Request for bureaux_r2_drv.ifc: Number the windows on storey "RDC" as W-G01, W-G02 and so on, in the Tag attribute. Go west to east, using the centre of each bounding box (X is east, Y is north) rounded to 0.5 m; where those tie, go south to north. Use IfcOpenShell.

First a look at what the model holds.

```python
import ifcopenshell
import ifcopenshell.util.element
import ifcopenshell.util.placement

model = ifcopenshell.open("bureaux_r2_drv.ifc")
print(model.schema)
storey = next(s for s in model.by_type("IfcBuildingStorey") if s.Name == "RDC")
windows = [e for e in ifcopenshell.util.element.get_decomposition(storey) if e.is_a("IfcWindow")]
for e in sorted(windows, key=lambda e: e.id()):
    origin = ifcopenshell.util.placement.get_local_placement(e.ObjectPlacement)[:3, 3]
    print(e.id(), e.Tag, e.Name, origin.round(2) + 0.0, sep=" | ")
```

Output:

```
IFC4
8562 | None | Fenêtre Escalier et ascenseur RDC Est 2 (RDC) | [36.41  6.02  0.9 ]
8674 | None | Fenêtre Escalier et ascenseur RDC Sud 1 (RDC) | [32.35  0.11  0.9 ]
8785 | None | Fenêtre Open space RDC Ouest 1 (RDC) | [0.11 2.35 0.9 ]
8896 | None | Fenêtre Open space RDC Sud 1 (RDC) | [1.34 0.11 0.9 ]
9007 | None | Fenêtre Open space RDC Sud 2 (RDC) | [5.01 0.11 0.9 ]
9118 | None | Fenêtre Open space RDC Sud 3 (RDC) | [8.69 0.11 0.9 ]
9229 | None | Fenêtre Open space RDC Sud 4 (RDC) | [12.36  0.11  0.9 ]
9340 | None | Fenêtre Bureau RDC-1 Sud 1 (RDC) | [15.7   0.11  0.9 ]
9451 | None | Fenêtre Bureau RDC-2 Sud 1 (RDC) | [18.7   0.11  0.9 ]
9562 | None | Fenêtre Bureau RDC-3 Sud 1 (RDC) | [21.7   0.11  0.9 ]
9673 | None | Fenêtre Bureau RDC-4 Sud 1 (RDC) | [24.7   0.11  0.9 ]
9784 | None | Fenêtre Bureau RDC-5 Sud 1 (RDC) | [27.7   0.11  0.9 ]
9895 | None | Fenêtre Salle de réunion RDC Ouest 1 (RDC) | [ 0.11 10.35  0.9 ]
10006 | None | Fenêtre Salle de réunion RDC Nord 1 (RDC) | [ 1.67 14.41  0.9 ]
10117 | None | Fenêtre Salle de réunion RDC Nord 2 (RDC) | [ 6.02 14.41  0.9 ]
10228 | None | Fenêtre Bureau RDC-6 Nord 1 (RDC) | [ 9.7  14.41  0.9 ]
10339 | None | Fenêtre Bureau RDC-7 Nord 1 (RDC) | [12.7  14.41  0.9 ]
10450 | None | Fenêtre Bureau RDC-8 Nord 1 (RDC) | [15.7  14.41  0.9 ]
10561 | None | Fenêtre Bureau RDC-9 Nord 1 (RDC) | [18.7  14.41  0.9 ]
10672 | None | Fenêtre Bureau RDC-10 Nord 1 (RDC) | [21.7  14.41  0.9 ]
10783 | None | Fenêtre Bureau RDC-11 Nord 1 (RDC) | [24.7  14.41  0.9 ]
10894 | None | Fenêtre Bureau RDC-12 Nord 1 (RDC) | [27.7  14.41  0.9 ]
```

```python
import ifcopenshell
import ifcopenshell.geom
import ifcopenshell.util.element
import ifcopenshell.util.shape

model = ifcopenshell.open("bureaux_r2_drv.ifc")
settings = ifcopenshell.geom.settings()
settings.set("use-world-coords", True)


def centre(element):
    shape = ifcopenshell.geom.create_shape(settings, element)
    return ifcopenshell.util.shape.get_bbox_centroid(shape.geometry)


storey = next(s for s in model.by_type("IfcBuildingStorey") if s.Name == "RDC")
windows = [e for e in ifcopenshell.util.element.get_decomposition(storey) if e.is_a("IfcWindow")]

# Insertion points can sit at a corner or the storey origin, so sort by the geometry (in metres).
centres = {e: centre(e) for e in windows}
windows.sort(key=lambda e: (round(centres[e][0] / 0.5), centres[e][1]))

for i, e in enumerate(windows, start=1):
    number = f"W-G{i:02d}"
    e.Tag = number
    print(e.id(), number)

model.write("bureaux_r2_drv-out.ifc")
```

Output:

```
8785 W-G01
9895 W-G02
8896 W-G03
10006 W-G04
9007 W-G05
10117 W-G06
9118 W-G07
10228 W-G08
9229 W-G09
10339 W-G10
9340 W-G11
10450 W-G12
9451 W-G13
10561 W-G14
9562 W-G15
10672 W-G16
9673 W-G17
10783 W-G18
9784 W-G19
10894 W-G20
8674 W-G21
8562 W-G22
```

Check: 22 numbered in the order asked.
